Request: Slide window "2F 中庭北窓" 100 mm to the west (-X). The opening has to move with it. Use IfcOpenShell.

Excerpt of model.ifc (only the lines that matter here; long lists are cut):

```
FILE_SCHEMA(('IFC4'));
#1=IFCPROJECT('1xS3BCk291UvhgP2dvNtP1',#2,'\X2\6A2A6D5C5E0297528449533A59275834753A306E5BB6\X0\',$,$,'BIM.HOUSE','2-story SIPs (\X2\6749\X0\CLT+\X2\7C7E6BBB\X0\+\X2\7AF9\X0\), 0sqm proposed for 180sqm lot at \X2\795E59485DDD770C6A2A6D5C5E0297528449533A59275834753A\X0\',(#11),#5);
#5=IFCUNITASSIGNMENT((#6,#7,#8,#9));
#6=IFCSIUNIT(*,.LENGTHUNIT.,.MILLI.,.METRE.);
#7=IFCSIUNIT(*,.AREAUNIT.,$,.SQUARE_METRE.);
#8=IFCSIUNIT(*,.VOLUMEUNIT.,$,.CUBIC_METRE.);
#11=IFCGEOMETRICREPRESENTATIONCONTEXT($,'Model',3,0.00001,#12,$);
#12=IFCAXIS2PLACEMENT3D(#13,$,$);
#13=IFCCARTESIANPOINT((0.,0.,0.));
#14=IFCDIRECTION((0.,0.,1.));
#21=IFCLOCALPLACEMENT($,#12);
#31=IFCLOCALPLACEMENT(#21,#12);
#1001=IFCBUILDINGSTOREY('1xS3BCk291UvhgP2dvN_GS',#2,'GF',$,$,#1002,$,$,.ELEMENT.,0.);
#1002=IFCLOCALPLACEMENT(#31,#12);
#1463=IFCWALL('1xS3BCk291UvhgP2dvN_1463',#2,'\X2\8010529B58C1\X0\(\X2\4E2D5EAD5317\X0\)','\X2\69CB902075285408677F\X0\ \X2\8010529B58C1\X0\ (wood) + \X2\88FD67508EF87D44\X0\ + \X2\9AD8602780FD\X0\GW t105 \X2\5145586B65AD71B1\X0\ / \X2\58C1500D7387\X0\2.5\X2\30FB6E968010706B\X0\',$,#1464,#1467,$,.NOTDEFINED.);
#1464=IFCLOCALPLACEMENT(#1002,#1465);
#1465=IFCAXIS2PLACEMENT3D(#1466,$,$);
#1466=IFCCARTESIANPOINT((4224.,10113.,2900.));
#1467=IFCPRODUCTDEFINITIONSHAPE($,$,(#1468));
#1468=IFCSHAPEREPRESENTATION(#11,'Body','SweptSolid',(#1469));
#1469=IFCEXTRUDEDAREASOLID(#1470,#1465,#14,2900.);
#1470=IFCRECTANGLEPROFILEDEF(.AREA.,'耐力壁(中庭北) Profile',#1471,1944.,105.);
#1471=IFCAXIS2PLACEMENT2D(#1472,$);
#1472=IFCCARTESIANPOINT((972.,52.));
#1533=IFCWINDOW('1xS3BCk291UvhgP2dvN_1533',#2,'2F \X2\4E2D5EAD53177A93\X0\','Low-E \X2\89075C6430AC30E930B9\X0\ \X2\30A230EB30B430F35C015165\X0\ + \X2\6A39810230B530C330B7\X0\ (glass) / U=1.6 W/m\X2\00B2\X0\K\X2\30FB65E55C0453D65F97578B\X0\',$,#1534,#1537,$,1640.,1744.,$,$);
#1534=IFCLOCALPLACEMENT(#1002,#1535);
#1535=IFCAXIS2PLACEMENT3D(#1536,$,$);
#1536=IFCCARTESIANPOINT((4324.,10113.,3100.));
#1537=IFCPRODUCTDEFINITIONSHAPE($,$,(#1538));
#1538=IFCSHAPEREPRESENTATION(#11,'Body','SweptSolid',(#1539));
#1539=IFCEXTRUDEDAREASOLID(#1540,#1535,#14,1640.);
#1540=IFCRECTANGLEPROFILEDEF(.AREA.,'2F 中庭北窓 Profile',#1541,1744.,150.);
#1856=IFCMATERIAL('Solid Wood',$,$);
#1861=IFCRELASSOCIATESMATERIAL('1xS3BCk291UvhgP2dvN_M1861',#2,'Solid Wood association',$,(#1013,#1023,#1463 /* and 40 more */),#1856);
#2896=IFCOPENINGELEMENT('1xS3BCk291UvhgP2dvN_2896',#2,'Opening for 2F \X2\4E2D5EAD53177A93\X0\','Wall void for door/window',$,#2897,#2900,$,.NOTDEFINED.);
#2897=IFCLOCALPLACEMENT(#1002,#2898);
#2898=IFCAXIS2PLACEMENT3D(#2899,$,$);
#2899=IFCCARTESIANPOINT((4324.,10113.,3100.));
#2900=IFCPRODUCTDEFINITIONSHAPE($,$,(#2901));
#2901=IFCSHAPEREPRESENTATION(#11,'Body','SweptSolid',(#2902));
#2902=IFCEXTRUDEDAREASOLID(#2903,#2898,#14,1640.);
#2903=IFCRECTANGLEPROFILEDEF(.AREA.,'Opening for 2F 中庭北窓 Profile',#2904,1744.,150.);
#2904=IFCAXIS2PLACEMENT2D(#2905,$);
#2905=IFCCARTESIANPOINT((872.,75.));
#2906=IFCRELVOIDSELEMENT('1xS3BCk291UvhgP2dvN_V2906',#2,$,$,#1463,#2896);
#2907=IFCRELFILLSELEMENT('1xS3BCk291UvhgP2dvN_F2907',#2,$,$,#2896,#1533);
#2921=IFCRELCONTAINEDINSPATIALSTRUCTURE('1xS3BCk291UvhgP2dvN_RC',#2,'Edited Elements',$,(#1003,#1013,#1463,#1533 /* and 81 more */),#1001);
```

```python
import ifcopenshell
import ifcopenshell.api.geometry
import ifcopenshell.util.placement
import ifcopenshell.util.unit

model = ifcopenshell.open("model.ifc")
unit_scale = ifcopenshell.util.unit.calculate_unit_scale(model)

window = model.by_id(1533)
opening = window.FillsVoids[0].RelatingOpeningElement
wall = opening.VoidsElements[0].RelatingBuildingElement

wall_matrix = ifcopenshell.util.placement.get_local_placement(wall.ObjectPlacement)
shift = wall_matrix[:3, 0] * -0.1 / unit_scale
before = ifcopenshell.util.placement.get_local_placement(window.ObjectPlacement)[:3, 3].copy()

# The window is not placed relative to its opening, so move both.
for product in (opening, window):
    matrix = ifcopenshell.util.placement.get_local_placement(product.ObjectPlacement)
    matrix[:3, 3] += shift
    ifcopenshell.api.geometry.edit_object_placement(model, product=product, matrix=matrix, is_si=False)

after = ifcopenshell.util.placement.get_local_placement(window.ObjectPlacement)[:3, 3]
print("window moved by", (after - before).round(3) + 0.0)

model.write("model_updated.ifc")
```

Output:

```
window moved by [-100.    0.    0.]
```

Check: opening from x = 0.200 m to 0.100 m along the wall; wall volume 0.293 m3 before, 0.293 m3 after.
